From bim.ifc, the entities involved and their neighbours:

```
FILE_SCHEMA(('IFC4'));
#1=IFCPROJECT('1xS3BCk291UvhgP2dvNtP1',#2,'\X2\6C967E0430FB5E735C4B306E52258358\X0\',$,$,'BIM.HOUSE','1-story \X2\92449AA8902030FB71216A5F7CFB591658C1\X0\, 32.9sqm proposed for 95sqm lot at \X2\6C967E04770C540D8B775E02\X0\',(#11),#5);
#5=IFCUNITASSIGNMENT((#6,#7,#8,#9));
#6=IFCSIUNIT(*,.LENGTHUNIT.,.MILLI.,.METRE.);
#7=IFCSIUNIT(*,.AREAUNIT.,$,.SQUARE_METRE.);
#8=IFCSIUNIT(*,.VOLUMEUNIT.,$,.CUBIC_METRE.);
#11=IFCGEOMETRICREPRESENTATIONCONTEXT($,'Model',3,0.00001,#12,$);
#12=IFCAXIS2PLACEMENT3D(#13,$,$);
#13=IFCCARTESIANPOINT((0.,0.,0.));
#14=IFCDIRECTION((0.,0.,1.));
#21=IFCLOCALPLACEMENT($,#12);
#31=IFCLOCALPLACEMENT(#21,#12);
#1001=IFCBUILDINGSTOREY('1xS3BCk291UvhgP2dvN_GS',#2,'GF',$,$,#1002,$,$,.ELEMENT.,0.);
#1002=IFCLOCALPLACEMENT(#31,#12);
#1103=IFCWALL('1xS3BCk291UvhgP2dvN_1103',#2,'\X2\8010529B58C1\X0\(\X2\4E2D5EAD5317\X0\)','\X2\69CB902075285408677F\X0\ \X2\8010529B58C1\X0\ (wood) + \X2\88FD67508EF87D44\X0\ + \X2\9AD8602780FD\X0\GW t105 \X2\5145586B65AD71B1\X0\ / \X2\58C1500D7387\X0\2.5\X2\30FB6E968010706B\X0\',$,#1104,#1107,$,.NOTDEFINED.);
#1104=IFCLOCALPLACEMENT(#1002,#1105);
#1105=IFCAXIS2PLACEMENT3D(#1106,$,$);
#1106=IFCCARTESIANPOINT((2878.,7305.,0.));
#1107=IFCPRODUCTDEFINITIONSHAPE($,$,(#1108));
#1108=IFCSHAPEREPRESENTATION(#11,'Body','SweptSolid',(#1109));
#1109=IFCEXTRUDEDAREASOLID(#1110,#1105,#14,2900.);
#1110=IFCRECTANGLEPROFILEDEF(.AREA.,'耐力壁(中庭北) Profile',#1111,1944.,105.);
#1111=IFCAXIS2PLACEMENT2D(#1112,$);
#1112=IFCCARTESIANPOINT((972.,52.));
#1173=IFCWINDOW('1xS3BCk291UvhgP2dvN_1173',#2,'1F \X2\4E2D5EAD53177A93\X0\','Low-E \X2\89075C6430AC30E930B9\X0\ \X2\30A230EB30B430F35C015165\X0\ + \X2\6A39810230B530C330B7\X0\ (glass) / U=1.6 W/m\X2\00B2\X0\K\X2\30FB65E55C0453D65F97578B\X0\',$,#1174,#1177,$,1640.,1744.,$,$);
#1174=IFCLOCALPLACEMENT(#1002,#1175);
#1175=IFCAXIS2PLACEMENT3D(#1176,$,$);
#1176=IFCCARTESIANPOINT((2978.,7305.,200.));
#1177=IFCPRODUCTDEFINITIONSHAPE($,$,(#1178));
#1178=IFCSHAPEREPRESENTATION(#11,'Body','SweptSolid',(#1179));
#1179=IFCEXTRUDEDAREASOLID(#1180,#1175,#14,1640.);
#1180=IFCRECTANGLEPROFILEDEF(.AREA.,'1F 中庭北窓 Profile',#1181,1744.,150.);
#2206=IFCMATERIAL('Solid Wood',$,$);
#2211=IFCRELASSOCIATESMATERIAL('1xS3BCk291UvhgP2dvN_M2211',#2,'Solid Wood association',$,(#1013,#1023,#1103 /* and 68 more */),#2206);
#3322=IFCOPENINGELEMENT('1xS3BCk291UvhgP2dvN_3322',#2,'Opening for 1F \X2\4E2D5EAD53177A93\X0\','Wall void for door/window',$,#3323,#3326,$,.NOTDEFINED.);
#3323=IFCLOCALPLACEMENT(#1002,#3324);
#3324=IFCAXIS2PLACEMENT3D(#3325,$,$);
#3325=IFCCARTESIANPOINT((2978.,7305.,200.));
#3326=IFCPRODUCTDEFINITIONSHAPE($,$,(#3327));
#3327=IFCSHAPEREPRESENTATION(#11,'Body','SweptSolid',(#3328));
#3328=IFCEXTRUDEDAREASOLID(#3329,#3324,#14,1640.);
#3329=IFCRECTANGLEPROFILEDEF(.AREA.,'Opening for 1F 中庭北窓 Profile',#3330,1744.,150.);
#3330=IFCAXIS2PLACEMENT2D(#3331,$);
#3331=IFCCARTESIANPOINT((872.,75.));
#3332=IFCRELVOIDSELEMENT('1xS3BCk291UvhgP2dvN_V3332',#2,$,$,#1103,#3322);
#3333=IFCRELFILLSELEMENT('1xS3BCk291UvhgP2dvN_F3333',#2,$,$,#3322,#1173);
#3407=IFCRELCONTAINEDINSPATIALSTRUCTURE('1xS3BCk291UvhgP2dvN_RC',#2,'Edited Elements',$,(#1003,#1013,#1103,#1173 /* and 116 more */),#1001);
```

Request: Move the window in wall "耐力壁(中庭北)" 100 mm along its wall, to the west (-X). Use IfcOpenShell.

```python
import ifcopenshell
import ifcopenshell.api.geometry
import ifcopenshell.util.placement
import ifcopenshell.util.unit

model = ifcopenshell.open("bim.ifc")
unit_scale = ifcopenshell.util.unit.calculate_unit_scale(model)

window = model.by_guid("1xS3BCk291UvhgP2dvN_1173")
opening = window.FillsVoids[0].RelatingOpeningElement
wall = opening.VoidsElements[0].RelatingBuildingElement

wall_matrix = ifcopenshell.util.placement.get_local_placement(wall.ObjectPlacement)
shift = wall_matrix[:3, 0] * -0.1 / unit_scale
before = ifcopenshell.util.placement.get_local_placement(window.ObjectPlacement)[:3, 3].copy()

# The window is not placed relative to its opening, so move both.
for product in (opening, window):
    matrix = ifcopenshell.util.placement.get_local_placement(product.ObjectPlacement)
    matrix[:3, 3] += shift
    ifcopenshell.api.geometry.edit_object_placement(model, product=product, matrix=matrix, is_si=False)

after = ifcopenshell.util.placement.get_local_placement(window.ObjectPlacement)[:3, 3]
print("window moved by", (after - before).round(3) + 0.0)

model.write("bim_edited.ifc")
```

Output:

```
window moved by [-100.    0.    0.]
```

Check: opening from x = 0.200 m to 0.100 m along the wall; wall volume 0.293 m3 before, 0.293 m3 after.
